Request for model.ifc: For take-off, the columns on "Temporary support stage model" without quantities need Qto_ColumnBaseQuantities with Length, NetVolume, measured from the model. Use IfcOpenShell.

First a look at what the model holds.

```python
import ifcopenshell
import ifcopenshell.util.element
import ifcopenshell.util.unit

model = ifcopenshell.open("model.ifc")
print(model.schema)
for unit_type in ("LENGTHUNIT", "AREAUNIT", "VOLUMEUNIT"):
    print(unit_type, ifcopenshell.util.unit.calculate_unit_scale(model, unit_type))
storey = next(s for s in model.by_type("IfcBuildingStorey") if s.Name == "Temporary support stage model")
columns = [e for e in ifcopenshell.util.element.get_decomposition(storey) if e.is_a("IfcColumn")]
for e in sorted(columns, key=lambda e: e.id()):
    print(e.id(), e.is_a(), e.Name, list(ifcopenshell.util.element.get_psets(e, qtos_only=True)), sep=" | ")
```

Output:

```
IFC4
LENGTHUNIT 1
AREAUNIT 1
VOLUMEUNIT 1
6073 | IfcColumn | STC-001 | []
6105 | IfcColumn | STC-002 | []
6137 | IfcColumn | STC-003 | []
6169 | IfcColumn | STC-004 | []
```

```python
import ifcopenshell
import ifcopenshell.api.pset
import ifcopenshell.geom
import ifcopenshell.util.element
import ifcopenshell.util.shape
import ifcopenshell.util.unit

model = ifcopenshell.open("model.ifc")
unit_scale = ifcopenshell.util.unit.calculate_unit_scale(model)
volume_scale = ifcopenshell.util.unit.calculate_unit_scale(model, "VOLUMEUNIT")
settings = ifcopenshell.geom.settings()

storey = next(s for s in model.by_type("IfcBuildingStorey") if s.Name == "Temporary support stage model")
columns = [e for e in ifcopenshell.util.element.get_decomposition(storey) if e.is_a("IfcColumn")]

for e in sorted(columns, key=lambda e: e.id()):
    if ifcopenshell.util.element.get_psets(e, qtos_only=True, should_inherit=False):
        continue
    # Geometry comes back in metres, in the element's own axes.
    shape = ifcopenshell.geom.create_shape(settings, e)
    values = {
        "Length": ifcopenshell.util.shape.get_z(shape.geometry) / unit_scale,
        "NetVolume": ifcopenshell.util.shape.get_volume(shape.geometry) / volume_scale,
    }
    qto = ifcopenshell.api.pset.add_qto(model, product=e, name="Qto_ColumnBaseQuantities")
    ifcopenshell.api.pset.edit_qto(model, qto=qto, properties=values)
    print(e.id(), {k: round(v, 3) for k, v in values.items()})

model.write("model_v2.ifc")
```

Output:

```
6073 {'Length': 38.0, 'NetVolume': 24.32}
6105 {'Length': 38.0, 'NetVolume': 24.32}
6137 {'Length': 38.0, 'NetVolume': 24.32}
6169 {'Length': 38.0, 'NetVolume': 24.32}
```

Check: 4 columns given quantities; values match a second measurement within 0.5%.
